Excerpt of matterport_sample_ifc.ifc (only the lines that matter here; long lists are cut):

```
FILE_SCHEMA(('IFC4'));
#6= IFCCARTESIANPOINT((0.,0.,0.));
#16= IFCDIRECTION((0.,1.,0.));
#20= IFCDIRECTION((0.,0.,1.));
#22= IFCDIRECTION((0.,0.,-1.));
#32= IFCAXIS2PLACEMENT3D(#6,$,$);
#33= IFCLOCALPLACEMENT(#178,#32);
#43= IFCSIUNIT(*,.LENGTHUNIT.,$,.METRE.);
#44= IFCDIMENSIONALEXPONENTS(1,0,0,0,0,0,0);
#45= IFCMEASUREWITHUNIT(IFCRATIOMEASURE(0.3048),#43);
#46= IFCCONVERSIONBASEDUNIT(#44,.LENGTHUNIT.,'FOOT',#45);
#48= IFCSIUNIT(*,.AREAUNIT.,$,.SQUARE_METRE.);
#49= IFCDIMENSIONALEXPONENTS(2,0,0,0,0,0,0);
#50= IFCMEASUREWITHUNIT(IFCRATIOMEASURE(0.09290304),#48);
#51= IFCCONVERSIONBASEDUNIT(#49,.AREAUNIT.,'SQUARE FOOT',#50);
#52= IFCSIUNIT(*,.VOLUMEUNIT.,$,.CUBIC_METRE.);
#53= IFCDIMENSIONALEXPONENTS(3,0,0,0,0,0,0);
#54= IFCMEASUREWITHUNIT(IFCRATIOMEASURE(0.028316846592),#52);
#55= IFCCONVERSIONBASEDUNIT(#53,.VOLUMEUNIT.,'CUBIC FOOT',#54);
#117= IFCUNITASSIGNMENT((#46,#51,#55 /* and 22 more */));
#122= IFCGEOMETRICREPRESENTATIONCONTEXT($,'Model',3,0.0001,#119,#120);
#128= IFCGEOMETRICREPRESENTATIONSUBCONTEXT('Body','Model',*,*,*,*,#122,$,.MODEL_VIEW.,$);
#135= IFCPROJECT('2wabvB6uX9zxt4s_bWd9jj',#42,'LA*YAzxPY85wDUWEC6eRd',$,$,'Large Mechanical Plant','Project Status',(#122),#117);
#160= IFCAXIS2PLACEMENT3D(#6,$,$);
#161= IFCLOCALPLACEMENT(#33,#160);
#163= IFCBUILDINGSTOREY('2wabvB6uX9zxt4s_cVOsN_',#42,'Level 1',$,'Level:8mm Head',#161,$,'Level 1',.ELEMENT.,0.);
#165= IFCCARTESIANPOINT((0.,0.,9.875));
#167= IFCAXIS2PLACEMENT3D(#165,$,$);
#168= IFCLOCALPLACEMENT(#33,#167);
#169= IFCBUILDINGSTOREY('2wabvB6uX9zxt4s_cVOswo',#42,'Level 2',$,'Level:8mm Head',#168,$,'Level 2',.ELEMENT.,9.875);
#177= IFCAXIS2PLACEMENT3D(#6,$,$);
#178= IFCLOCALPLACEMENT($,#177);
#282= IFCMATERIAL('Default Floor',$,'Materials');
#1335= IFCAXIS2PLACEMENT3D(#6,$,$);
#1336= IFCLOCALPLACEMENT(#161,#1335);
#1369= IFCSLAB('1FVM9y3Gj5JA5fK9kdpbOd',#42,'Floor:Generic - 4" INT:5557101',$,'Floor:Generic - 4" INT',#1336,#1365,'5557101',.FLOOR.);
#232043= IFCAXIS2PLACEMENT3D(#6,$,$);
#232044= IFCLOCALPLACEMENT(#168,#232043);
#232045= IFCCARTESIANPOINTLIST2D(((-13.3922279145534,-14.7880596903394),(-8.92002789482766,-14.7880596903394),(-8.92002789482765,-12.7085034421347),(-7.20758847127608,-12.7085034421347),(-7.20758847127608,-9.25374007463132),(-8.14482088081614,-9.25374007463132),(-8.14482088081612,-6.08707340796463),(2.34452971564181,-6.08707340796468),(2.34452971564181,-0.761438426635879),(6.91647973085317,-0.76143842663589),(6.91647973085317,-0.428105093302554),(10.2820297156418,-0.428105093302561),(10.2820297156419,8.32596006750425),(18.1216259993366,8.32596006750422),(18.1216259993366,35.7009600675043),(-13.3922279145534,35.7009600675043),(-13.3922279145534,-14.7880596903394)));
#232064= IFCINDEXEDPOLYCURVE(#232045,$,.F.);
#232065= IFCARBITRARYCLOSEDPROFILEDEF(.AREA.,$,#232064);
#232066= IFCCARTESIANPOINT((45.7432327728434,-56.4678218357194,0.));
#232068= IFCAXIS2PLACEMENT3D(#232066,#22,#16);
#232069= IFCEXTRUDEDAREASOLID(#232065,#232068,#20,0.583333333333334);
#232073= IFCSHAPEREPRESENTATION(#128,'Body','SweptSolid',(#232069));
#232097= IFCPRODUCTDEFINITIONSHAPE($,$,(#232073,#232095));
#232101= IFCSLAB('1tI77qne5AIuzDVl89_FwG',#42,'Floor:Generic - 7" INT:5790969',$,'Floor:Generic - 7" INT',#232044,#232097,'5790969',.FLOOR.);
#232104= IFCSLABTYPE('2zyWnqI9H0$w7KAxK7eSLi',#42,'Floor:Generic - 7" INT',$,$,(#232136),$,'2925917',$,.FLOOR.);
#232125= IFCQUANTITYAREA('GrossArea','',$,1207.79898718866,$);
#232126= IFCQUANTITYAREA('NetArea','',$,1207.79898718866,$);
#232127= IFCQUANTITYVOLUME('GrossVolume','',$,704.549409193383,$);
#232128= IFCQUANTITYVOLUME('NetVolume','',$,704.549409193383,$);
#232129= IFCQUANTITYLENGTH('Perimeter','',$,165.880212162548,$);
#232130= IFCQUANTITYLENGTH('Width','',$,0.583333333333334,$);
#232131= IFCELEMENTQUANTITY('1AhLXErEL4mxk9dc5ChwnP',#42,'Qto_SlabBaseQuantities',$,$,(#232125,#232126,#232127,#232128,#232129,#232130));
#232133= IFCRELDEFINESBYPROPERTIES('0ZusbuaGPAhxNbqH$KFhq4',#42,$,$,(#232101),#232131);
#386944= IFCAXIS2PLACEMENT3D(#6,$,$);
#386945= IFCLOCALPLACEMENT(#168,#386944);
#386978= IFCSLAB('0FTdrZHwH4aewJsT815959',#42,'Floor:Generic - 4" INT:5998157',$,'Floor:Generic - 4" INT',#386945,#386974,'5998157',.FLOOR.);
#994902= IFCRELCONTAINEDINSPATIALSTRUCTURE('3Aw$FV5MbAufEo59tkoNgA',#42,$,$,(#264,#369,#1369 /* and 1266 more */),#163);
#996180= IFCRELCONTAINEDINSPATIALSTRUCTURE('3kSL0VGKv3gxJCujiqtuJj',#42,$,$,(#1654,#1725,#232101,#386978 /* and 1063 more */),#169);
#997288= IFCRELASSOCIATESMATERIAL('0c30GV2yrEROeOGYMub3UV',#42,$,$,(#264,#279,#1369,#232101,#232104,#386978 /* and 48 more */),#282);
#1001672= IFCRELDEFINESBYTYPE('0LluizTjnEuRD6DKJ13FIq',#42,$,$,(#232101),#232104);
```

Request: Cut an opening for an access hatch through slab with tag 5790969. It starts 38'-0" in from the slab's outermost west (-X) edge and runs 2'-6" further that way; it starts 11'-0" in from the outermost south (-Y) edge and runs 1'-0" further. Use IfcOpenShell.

```python
import numpy as np
import ifcopenshell
import ifcopenshell.api.feature
import ifcopenshell.api.geometry
import ifcopenshell.api.pset
import ifcopenshell.api.root
import ifcopenshell.geom
import ifcopenshell.util.element
import ifcopenshell.util.placement
import ifcopenshell.util.representation
import ifcopenshell.util.shape
import ifcopenshell.util.unit

model = ifcopenshell.open("matterport_sample_ifc.ifc")
unit_scale = ifcopenshell.util.unit.calculate_unit_scale(model)
area_scale = ifcopenshell.util.unit.calculate_unit_scale(model, "AREAUNIT")
volume_scale = ifcopenshell.util.unit.calculate_unit_scale(model, "VOLUMEUNIT")
settings = ifcopenshell.geom.settings()


def volume(element):
    """Net volume in cubic metres, openings subtracted."""
    shape = ifcopenshell.geom.create_shape(settings, element)
    return ifcopenshell.util.shape.get_volume(shape.geometry)


slab = model.by_guid("1tI77qne5AIuzDVl89_FwG")
before = volume(slab)

# Extent in the slab's own axes, in metres. The edges named are its -X and -Y sides.
slab_shape = ifcopenshell.geom.create_shape(settings, slab)
vertices = ifcopenshell.util.shape.get_vertices(slab_shape.geometry)
x_min, y_min, bottom = vertices.min(axis=0)
top = vertices[:, 2].max()

opening = ifcopenshell.api.root.create_entity(model, ifc_class="IfcOpeningElement", name="Access hatch opening", predefined_type="OPENING")
context = ifcopenshell.util.representation.get_context(model, "Model", "Body", "MODEL_VIEW")
width, depth = 0.762, 0.3048
outline = [(0.0, 0.0), (width, 0.0), (width, depth), (0.0, depth), (0.0, 0.0)]
# Overshoot both faces by 50 mm so the cut is clean.
shape = ifcopenshell.api.geometry.add_slab_representation(
    model, context=context, depth=top - bottom + 0.1, polyline=outline
)
ifcopenshell.api.geometry.assign_representation(model, product=opening, representation=shape)

matrix = ifcopenshell.util.placement.get_local_placement(slab.ObjectPlacement)
matrix[:, 3] = matrix @ np.append(np.array([x_min + 11.5824, y_min + 3.3528, bottom - 0.05]) / unit_scale, 1.0)
ifcopenshell.api.geometry.edit_object_placement(model, product=opening, matrix=matrix, is_si=False)
ifcopenshell.api.feature.add_feature(model, feature=opening, element=slab)

after = volume(slab)

# Update the slab's stored quantities.
qto = model.by_id(ifcopenshell.util.element.get_pset(slab, "Qto_SlabBaseQuantities", should_inherit=False)["id"])
ifcopenshell.api.pset.edit_qto(model, qto=qto, properties={
    "NetArea": after / (top - bottom) / area_scale,
    "NetVolume": after / volume_scale,
})

print(f"slab volume {before:.3f} -> {after:.3f} m3")

model.write("matterport_sample_ifc_updated.ifc")
```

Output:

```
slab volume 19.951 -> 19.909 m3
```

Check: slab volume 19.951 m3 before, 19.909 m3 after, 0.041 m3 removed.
